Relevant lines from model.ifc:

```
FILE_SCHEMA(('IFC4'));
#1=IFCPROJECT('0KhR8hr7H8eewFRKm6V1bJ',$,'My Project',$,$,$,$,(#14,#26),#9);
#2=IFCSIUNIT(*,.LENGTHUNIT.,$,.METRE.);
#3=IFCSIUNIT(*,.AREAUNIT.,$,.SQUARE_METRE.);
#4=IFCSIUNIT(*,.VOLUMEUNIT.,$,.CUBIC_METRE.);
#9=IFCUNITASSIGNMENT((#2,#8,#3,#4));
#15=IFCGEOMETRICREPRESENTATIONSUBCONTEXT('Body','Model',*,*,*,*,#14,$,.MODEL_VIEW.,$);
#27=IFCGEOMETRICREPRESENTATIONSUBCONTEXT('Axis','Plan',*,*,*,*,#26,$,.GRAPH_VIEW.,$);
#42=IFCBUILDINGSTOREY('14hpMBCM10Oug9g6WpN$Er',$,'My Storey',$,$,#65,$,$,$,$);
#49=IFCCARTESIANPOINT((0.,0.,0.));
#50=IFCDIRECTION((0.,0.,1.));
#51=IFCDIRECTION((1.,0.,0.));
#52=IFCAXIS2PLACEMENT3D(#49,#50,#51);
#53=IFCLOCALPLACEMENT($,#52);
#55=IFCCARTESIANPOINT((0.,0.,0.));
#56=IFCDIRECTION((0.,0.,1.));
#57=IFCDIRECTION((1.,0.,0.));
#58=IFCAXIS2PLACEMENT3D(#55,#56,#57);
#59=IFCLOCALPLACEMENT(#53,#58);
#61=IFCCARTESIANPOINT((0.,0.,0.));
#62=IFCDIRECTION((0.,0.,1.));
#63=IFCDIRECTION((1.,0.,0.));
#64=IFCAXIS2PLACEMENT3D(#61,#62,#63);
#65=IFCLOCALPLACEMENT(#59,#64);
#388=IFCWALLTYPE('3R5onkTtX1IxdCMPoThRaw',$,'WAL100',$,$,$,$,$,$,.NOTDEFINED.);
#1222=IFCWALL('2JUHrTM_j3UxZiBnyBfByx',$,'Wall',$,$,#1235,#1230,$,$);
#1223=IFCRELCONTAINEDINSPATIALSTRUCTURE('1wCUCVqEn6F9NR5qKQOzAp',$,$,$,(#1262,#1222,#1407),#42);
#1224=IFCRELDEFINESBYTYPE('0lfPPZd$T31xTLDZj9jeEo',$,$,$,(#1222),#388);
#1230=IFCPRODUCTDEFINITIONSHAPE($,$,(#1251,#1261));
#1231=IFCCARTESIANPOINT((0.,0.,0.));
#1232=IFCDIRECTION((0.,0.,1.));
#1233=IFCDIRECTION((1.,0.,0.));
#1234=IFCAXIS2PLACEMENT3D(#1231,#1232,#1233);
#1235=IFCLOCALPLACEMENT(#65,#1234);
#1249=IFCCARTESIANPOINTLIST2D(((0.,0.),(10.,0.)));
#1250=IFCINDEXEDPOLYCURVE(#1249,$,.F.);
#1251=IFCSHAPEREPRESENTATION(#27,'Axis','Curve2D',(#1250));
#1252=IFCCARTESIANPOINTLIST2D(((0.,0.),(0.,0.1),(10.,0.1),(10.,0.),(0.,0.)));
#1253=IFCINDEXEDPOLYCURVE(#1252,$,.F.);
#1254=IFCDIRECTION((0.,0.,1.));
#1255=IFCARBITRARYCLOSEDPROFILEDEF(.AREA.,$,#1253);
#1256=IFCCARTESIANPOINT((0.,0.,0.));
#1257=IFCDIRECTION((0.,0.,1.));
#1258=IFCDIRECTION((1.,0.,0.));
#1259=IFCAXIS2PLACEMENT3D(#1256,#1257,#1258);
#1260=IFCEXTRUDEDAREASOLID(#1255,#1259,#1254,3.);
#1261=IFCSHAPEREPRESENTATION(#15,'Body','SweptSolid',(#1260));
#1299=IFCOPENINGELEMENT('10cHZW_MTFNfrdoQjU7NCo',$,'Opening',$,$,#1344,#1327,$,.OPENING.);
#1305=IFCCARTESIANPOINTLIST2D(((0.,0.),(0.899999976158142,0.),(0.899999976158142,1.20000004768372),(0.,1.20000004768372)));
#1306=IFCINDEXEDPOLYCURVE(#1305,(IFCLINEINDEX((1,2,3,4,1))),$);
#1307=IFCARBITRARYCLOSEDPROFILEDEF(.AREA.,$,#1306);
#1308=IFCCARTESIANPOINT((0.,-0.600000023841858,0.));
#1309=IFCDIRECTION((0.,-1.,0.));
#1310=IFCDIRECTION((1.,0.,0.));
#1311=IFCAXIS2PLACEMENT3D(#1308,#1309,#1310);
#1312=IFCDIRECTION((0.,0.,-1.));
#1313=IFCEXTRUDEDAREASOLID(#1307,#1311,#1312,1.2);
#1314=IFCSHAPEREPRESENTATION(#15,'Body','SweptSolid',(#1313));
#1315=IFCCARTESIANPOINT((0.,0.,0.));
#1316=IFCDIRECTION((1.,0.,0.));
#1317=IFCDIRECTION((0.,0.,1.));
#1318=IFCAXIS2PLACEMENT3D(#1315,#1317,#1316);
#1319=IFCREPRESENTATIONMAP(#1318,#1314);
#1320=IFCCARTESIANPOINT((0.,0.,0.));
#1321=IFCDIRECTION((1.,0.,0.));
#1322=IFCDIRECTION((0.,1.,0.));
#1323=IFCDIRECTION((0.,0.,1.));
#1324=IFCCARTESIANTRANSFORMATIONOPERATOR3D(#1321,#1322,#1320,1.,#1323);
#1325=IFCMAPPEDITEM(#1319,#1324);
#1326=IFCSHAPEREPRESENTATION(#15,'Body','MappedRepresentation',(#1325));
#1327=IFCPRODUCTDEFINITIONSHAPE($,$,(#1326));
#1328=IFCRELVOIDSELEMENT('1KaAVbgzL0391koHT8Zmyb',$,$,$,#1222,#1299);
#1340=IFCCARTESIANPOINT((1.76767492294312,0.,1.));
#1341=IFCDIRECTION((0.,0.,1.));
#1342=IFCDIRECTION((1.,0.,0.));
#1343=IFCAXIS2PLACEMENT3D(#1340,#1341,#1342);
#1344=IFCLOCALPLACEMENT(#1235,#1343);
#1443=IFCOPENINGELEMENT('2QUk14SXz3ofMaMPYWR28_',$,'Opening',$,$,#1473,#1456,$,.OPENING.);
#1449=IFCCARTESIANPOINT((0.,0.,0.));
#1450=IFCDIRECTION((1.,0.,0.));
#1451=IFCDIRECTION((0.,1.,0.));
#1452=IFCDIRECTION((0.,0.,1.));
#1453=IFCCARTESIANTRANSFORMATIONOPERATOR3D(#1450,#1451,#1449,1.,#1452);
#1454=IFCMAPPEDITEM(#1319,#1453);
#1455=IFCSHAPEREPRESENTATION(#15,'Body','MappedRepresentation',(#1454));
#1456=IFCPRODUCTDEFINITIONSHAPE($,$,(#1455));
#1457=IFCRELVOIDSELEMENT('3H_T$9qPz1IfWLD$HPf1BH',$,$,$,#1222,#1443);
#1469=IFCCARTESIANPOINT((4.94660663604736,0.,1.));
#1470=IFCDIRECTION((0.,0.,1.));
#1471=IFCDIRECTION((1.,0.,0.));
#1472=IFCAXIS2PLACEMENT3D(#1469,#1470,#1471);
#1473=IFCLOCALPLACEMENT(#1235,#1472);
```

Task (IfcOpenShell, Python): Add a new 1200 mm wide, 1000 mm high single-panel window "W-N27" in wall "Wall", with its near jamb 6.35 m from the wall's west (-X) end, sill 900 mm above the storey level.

```python
import numpy as np
import ifcopenshell
import ifcopenshell.api.feature
import ifcopenshell.api.geometry
import ifcopenshell.api.root
import ifcopenshell.api.spatial
import ifcopenshell.geom
import ifcopenshell.util.element
import ifcopenshell.util.placement
import ifcopenshell.util.representation
import ifcopenshell.util.shape
import ifcopenshell.util.unit

model = ifcopenshell.open("model.ifc")
unit_scale = ifcopenshell.util.unit.calculate_unit_scale(model)
settings = ifcopenshell.geom.settings()


def volume(element):
    """Net volume in cubic metres, openings subtracted."""
    shape = ifcopenshell.geom.create_shape(settings, element)
    return ifcopenshell.util.shape.get_volume(shape.geometry)


wall = model.by_guid("2JUHrTM_j3UxZiBnyBfByx")
storey = ifcopenshell.util.element.get_container(wall, ifc_class="IfcBuildingStorey")
context = ifcopenshell.util.representation.get_context(model, "Model", "Body", "MODEL_VIEW")
before = volume(wall)

width, height, from_end, sill = 1.2, 1, 6.35, 0.9  # metres

# The wall runs along its own X axis, and the end named is its -X end.
wall_shape = ifcopenshell.geom.create_shape(settings, wall)
x, y, z = ifcopenshell.util.shape.get_vertices(wall_shape.geometry).T
start = x.min() + from_end
face, thickness = float(y.min()), float(y.max() - y.min())
wall_matrix = ifcopenshell.util.placement.get_local_placement(wall.ObjectPlacement)
level = ifcopenshell.util.placement.get_local_placement(storey.ObjectPlacement)[2, 3]


def in_wall(x, y):
    """Placement at x, y metres in the wall's axes, at sill height."""
    matrix = wall_matrix.copy()
    matrix[:, 3] = wall_matrix @ np.array([x / unit_scale, y / unit_scale, 0.0, 1.0])
    matrix[2, 3] = level + sill / unit_scale
    return matrix


# Opening: a box that overshoots both wall faces by 50 mm.
opening = ifcopenshell.api.root.create_entity(model, ifc_class="IfcOpeningElement", predefined_type="OPENING")
box = ifcopenshell.api.geometry.add_wall_representation(
    model, context=context, length=width, height=height, thickness=thickness + 0.1
)
ifcopenshell.api.geometry.assign_representation(model, product=opening, representation=box)
ifcopenshell.api.geometry.edit_object_placement(model, product=opening, matrix=in_wall(start, face - 0.05), is_si=False)
ifcopenshell.api.feature.add_feature(model, feature=opening, element=wall)

window = ifcopenshell.api.root.create_entity(model, ifc_class="IfcWindow", name="W-N27", predefined_type="WINDOW")
window.OverallWidth, window.OverallHeight = width / unit_scale, height / unit_scale
window.PartitioningType = "SINGLE_PANEL"
body = ifcopenshell.api.geometry.add_window_representation(
    model,
    context=context,
    overall_width=window.OverallWidth,
    overall_height=window.OverallHeight,
    partition_type="SINGLE_PANEL",
)
ifcopenshell.api.geometry.assign_representation(model, product=window, representation=body)
ifcopenshell.api.spatial.assign_container(model, products=[window], relating_structure=storey)
ifcopenshell.api.feature.add_filling(model, opening=opening, element=window)

# Centre the window in the wall's thickness.
ifcopenshell.api.geometry.edit_object_placement(model, product=window, matrix=in_wall(start, face), is_si=False)
window_shape = ifcopenshell.geom.create_shape(settings, window)
depth = ifcopenshell.util.shape.get_vertices(window_shape.geometry)[:, 1]
offset = face + thickness / 2 - (depth.min() + depth.max()) / 2
ifcopenshell.api.geometry.edit_object_placement(model, product=window, matrix=in_wall(start, offset), is_si=False)

after = volume(wall)

print(f"wall volume {before:.3f} -> {after:.3f} m3")

model.write("model_v2.ifc")
```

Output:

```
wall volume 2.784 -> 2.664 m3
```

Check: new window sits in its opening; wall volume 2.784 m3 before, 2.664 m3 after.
